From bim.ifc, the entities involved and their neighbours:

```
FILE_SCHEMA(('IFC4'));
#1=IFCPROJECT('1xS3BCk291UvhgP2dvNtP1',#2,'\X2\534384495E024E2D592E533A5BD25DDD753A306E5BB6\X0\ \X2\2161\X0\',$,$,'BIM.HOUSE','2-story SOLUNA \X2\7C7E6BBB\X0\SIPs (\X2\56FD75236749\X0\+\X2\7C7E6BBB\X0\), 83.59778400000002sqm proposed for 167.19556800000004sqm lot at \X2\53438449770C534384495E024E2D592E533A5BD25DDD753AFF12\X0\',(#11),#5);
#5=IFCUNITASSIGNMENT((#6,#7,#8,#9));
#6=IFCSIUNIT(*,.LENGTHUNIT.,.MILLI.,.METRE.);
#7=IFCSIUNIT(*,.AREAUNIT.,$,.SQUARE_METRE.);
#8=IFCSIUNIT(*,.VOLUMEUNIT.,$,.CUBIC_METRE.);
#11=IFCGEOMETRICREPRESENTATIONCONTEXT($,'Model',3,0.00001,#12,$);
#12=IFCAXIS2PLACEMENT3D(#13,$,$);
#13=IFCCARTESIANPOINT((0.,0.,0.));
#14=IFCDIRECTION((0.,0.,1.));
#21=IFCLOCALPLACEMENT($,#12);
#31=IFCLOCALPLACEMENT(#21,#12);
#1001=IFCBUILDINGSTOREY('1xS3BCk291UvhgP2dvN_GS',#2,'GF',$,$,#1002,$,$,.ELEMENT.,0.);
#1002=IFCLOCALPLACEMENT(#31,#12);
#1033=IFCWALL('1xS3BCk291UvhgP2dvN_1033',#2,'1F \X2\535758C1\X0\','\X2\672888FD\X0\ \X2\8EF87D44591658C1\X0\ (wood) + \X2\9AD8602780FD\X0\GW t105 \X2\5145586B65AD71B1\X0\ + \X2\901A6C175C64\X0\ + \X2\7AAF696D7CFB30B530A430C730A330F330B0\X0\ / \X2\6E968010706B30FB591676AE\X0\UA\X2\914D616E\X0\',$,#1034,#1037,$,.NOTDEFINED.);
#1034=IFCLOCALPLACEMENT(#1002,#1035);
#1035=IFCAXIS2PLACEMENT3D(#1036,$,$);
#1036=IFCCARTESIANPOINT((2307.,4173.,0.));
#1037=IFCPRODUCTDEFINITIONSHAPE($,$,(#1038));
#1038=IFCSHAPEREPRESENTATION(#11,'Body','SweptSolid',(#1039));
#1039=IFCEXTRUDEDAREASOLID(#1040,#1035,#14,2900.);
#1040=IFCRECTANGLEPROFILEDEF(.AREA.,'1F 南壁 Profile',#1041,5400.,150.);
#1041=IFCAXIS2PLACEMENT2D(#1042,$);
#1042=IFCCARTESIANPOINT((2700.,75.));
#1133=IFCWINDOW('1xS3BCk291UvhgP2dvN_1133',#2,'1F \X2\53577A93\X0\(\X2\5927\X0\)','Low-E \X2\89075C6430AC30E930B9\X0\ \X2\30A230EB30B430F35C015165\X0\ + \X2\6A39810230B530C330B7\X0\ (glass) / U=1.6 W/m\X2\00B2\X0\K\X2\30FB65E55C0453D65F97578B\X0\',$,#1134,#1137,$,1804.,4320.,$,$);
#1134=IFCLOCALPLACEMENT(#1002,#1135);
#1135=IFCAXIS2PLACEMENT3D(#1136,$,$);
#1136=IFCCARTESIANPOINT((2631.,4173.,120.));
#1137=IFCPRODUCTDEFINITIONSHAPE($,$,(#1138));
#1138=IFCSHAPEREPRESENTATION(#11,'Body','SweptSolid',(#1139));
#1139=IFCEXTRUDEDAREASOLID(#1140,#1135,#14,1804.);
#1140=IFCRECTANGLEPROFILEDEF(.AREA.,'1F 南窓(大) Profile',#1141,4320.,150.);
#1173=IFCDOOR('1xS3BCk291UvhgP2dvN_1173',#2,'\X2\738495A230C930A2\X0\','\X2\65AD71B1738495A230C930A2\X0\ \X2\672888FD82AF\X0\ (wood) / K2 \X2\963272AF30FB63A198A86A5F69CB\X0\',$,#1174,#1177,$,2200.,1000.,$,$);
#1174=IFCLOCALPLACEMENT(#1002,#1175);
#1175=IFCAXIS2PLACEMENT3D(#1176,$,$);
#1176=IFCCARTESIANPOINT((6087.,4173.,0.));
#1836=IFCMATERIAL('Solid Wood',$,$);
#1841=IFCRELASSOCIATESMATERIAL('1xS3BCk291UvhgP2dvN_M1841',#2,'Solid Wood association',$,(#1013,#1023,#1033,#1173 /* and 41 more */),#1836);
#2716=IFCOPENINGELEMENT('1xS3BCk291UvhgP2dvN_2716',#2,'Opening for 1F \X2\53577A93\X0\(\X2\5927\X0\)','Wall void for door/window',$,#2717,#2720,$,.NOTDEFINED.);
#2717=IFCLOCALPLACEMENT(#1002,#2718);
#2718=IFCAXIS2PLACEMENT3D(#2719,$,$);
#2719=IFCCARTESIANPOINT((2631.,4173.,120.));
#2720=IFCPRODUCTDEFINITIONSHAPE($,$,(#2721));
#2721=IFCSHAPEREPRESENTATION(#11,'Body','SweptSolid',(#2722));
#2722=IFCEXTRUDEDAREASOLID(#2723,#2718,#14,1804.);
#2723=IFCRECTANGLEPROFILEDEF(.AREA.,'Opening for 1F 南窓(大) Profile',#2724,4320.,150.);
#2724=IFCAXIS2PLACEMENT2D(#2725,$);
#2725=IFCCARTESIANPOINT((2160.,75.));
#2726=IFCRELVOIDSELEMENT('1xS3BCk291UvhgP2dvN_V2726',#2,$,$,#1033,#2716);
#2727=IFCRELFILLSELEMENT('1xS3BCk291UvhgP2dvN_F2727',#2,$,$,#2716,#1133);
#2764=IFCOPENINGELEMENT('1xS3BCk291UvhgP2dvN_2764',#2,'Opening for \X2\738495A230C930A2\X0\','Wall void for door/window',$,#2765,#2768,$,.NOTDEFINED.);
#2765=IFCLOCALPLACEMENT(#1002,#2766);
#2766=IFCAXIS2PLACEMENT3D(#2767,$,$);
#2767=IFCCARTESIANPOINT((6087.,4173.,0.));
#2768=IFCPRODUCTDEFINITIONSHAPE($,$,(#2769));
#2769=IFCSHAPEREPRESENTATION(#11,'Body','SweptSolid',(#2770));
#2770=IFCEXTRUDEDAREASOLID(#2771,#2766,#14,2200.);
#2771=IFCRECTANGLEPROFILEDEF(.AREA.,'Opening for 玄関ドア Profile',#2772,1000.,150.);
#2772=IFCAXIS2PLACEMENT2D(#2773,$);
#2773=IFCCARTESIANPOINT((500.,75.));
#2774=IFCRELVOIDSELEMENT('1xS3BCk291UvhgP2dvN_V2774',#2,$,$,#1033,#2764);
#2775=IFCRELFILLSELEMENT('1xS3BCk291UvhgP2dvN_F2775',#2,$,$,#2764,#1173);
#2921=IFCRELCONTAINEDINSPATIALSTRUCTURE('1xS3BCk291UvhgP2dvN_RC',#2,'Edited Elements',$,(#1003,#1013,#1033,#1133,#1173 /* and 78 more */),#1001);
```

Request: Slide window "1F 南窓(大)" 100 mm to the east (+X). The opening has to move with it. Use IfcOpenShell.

```python
import ifcopenshell
import ifcopenshell.api.geometry
import ifcopenshell.util.placement
import ifcopenshell.util.unit

model = ifcopenshell.open("bim.ifc")
unit_scale = ifcopenshell.util.unit.calculate_unit_scale(model)

window = model.by_id(1133)
opening = window.FillsVoids[0].RelatingOpeningElement
wall = opening.VoidsElements[0].RelatingBuildingElement

wall_matrix = ifcopenshell.util.placement.get_local_placement(wall.ObjectPlacement)
shift = wall_matrix[:3, 0] * 0.1 / unit_scale
before = ifcopenshell.util.placement.get_local_placement(window.ObjectPlacement)[:3, 3].copy()

# The window is not placed relative to its opening, so move both.
for product in (opening, window):
    matrix = ifcopenshell.util.placement.get_local_placement(product.ObjectPlacement)
    matrix[:3, 3] += shift
    ifcopenshell.api.geometry.edit_object_placement(model, product=product, matrix=matrix, is_si=False)

after = ifcopenshell.util.placement.get_local_placement(window.ObjectPlacement)[:3, 3]
print("window moved by", (after - before).round(3) + 0.0)

model.write("bim_edited.ifc")
```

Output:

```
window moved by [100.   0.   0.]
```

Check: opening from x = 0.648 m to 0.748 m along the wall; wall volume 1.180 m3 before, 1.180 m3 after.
